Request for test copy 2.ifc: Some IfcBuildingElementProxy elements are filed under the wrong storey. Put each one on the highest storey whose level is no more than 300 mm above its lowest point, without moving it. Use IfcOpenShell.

First a look at what the model holds.

```python
import ifcopenshell
import ifcopenshell.util.element
import ifcopenshell.util.placement

model = ifcopenshell.open("test copy 2.ifc")
print(model.schema)
for storey in model.by_type("IfcBuildingStorey"):
    level = ifcopenshell.util.placement.get_storey_elevation(storey)
    count = sum(e.is_a("IfcBuildingElementProxy") for e in ifcopenshell.util.element.get_contained(storey))
    print(storey.id(), storey.Name, round(level, 3), count, sep=" | ")
```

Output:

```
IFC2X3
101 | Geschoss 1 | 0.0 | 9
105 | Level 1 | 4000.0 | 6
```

```python
import ifcopenshell
import ifcopenshell.api.spatial
import ifcopenshell.geom
import ifcopenshell.util.element
import ifcopenshell.util.placement
import ifcopenshell.util.shape
import ifcopenshell.util.unit

model = ifcopenshell.open("test copy 2.ifc")
unit_scale = ifcopenshell.util.unit.calculate_unit_scale(model)
settings = ifcopenshell.geom.settings()

levels = sorted(
    ((ifcopenshell.util.placement.get_storey_elevation(s) * unit_scale, s) for s in model.by_type("IfcBuildingStorey")),
    key=lambda pair: pair[0],
)

for e in model.by_type("IfcBuildingElementProxy"):
    current = e.ContainedInStructure[0].RelatingStructure if e.ContainedInStructure else None
    if current is None or not current.is_a("IfcBuildingStorey"):
        continue
    shape = ifcopenshell.geom.create_shape(settings, e)
    bottom = ifcopenshell.util.shape.get_shape_bottom_elevation(shape, shape.geometry)
    below = [s for level, s in levels if level <= bottom + 0.3]
    storey = below[-1] if below else levels[0][1]
    if storey != current:
        # assign_container keeps the world position.
        ifcopenshell.api.spatial.assign_container(model, products=[e], relating_structure=storey)
        print(e.id(), current.Name, "->", storey.Name)

model.write("test copy 2_edited.ifc")
```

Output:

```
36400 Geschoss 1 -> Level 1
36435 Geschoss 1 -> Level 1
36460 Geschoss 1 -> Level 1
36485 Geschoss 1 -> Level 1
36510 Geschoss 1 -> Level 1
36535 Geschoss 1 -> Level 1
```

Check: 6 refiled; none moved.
